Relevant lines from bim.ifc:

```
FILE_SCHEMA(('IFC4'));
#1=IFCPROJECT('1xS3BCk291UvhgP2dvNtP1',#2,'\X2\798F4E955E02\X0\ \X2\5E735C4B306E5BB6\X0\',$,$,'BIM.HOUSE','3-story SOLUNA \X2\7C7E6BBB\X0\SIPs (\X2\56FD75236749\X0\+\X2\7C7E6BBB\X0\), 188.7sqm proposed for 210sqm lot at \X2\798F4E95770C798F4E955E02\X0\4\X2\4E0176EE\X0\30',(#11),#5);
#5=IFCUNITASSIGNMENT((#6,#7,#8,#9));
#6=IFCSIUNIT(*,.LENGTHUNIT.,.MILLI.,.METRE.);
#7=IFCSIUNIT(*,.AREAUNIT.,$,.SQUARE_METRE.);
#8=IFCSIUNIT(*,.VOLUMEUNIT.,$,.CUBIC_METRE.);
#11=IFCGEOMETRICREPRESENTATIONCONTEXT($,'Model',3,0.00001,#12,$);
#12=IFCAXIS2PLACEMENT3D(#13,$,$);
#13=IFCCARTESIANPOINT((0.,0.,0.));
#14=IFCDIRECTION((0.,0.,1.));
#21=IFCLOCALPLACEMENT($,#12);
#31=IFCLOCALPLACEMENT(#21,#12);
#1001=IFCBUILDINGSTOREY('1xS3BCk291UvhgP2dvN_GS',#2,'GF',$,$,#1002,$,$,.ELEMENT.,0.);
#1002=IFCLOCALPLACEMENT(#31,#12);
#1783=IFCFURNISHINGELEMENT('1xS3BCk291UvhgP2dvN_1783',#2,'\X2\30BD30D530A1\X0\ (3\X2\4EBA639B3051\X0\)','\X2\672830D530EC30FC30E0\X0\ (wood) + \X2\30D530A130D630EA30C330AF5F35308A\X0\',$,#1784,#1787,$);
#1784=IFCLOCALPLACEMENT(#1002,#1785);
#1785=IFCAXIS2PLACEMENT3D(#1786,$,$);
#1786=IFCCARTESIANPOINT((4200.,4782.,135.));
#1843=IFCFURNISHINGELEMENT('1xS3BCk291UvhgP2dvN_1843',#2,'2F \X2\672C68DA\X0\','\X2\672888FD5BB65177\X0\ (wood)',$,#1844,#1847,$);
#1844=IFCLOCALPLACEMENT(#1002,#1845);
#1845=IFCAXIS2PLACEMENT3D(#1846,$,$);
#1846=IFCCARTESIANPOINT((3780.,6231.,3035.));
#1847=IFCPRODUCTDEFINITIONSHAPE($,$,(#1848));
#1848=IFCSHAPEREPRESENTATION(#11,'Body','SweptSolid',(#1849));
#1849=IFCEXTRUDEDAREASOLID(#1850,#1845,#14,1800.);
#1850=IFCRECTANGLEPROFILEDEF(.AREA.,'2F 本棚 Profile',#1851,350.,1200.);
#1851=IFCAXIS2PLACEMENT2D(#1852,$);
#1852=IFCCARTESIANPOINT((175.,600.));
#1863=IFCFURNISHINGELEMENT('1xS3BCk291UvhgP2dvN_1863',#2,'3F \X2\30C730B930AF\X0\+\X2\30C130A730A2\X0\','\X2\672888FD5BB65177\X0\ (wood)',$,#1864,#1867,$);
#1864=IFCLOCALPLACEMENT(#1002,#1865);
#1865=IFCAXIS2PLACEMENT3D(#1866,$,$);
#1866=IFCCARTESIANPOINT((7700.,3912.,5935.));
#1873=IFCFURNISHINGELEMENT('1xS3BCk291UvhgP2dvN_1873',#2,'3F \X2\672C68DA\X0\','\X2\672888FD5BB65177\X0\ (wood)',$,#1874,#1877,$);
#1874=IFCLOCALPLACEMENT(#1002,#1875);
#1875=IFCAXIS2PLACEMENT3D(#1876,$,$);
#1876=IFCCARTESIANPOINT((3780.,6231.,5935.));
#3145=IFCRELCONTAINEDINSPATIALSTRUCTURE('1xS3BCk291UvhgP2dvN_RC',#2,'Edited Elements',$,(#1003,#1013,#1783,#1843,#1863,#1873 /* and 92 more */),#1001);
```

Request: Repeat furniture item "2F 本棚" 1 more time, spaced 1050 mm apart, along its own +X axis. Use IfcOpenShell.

```python
import ifcopenshell
import ifcopenshell.api.geometry
import ifcopenshell.api.root
import ifcopenshell.util.element
import ifcopenshell.util.placement
import ifcopenshell.util.unit

model = ifcopenshell.open("bim.ifc")
unit_scale = ifcopenshell.util.unit.calculate_unit_scale(model)


def reuse_history(source, copy):
    """copy_class also copies each property set's owner history, people and application; keep the originals."""
    for rel in copy.IsDefinedBy:
        if rel.is_a("IfcRelDefinesByProperties") and (history := rel.RelatingPropertyDefinition.OwnerHistory):
            rel.RelatingPropertyDefinition.OwnerHistory = source.OwnerHistory
            ifcopenshell.util.element.remove_deep2(model, history)


source = model.by_guid("1xS3BCk291UvhgP2dvN_1843")
base = ifcopenshell.util.placement.get_local_placement(source.ObjectPlacement)
step = base[:3, 0] * 1.05 / unit_scale

for i in range(1, 2):
    copy = ifcopenshell.api.root.copy_class(model, product=source)
    copy.Representation = ifcopenshell.util.element.copy_deep(
        model, source.Representation, exclude=["IfcGeometricRepresentationContext", "IfcRepresentationMap"]
    )
    reuse_history(source, copy)
    matrix = base.copy()
    matrix[:3, 3] += i * step
    print("added at", matrix[:3, 3].round(3) + 0.0)
    ifcopenshell.api.geometry.edit_object_placement(model, product=copy, matrix=matrix, is_si=False)

model.write("bim_updated.ifc")
```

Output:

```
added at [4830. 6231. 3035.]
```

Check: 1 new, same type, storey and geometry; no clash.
